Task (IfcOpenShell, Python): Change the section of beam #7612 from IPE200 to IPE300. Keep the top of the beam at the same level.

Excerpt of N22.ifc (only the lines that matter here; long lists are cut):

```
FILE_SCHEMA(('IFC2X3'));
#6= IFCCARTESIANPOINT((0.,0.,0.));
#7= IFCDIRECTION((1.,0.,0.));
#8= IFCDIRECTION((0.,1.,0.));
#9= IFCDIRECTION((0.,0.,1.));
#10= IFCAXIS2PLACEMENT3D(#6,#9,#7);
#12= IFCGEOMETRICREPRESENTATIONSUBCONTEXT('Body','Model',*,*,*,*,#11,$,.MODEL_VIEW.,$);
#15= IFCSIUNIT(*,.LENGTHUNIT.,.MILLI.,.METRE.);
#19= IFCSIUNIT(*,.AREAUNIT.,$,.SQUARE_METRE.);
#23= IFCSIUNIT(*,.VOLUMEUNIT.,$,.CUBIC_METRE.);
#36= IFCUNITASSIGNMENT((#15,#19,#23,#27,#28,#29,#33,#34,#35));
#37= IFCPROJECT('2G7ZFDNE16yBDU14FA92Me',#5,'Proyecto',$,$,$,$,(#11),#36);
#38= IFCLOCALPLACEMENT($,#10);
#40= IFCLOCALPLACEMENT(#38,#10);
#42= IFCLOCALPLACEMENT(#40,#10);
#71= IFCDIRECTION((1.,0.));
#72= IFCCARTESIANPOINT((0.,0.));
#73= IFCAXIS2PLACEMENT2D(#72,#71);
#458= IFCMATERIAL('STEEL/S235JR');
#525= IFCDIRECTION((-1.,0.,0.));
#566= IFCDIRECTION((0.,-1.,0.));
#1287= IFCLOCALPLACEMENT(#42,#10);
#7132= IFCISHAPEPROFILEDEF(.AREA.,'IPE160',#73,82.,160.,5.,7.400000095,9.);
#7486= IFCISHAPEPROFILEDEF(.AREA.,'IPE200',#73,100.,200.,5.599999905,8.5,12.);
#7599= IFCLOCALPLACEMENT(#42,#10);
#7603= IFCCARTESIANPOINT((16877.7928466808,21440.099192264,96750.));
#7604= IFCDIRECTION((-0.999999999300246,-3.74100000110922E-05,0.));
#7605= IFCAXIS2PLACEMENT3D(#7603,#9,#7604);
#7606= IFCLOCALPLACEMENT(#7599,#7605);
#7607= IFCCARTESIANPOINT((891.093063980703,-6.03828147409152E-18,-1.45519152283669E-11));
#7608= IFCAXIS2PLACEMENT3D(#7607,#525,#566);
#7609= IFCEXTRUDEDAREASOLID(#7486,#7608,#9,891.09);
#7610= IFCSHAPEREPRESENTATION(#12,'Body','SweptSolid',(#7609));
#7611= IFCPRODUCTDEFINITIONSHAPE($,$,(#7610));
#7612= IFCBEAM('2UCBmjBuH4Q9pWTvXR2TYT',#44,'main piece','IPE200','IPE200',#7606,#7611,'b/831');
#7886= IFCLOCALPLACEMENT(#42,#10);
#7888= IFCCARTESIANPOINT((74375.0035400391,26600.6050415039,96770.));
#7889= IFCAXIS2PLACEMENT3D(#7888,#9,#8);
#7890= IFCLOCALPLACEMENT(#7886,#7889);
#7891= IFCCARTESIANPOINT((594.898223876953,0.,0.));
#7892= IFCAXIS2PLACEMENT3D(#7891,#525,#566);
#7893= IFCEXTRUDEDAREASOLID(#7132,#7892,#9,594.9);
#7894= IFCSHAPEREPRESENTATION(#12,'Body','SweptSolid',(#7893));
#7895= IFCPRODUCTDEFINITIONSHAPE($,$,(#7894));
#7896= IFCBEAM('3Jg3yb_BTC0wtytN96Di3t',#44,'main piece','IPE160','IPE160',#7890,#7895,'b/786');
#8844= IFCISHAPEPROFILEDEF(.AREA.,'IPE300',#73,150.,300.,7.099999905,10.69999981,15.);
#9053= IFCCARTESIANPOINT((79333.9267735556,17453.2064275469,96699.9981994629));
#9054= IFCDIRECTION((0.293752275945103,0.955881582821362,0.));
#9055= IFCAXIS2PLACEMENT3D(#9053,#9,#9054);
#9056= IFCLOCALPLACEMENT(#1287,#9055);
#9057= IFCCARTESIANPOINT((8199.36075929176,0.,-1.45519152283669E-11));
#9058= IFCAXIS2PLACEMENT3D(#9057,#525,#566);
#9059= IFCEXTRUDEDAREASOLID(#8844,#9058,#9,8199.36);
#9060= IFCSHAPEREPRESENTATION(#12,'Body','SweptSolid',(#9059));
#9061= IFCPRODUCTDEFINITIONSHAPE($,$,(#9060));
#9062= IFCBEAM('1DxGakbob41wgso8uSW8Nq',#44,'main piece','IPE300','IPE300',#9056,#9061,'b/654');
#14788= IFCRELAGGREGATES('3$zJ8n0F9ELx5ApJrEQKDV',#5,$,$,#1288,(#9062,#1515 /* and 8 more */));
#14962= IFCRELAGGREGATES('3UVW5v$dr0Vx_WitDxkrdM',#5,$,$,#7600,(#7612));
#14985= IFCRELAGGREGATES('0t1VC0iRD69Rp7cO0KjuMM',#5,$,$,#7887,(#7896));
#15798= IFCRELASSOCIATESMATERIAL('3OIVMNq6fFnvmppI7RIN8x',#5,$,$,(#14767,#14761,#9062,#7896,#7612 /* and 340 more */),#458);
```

```python
import ifcopenshell
import ifcopenshell.util.element
import ifcopenshell.util.representation

model = ifcopenshell.open("N22.ifc")

member = model.by_guid("2UCBmjBuH4Q9pWTvXR2TYT")
source = next(p for p in model.by_type("IfcIShapeProfileDef") if p.ProfileName == "IPE300")

body = ifcopenshell.util.representation.get_representation(member, "Model", "Body")
solid = body.Items[0]
old_profile = solid.SweptArea

# Copy the section's sizes but keep this member's own profile position.
profile = ifcopenshell.util.element.copy(model, source)
# Profiles are centred, so shift by half the change in depth to hold the top.
shift = (old_profile.OverallDepth - profile.OverallDepth) / 2
x, y = old_profile.Position.Location.Coordinates
up = (0.0, 1.0)  # upwards, in the solid's own plane
location = model.createIfcCartesianPoint((x + up[0] * shift, y + up[1] * shift))
profile.Position = model.createIfcAxis2Placement2D(location, old_profile.Position.RefDirection)
solid.SweptArea = profile
if not model.get_total_inverses(old_profile):
    ifcopenshell.util.element.remove_deep2(model, old_profile)
member.Description = member.Description.replace("IPE200", "IPE300")
member.ObjectType = member.ObjectType.replace("IPE200", "IPE300")

print(solid.SweptArea)

model.write("N22_v2.ifc")
```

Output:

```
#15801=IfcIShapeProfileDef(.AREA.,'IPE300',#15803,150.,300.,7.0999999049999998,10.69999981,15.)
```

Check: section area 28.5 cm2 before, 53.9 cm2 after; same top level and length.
